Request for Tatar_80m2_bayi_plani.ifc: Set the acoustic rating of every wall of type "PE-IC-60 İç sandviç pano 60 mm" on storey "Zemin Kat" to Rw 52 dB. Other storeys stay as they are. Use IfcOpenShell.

First a look at what the model holds.

```python
import ifcopenshell
import ifcopenshell.util.element

model = ifcopenshell.open("Tatar_80m2_bayi_plani.ifc")
print(model.schema)
storey = next(s for s in model.by_type("IfcBuildingStorey") if s.Name == "Zemin Kat")
walls = [e for e in ifcopenshell.util.element.get_decomposition(storey) if e.is_a("IfcWall")]
seen = {}
for e in walls:
    element_type = ifcopenshell.util.element.get_type(e)
    key = (element_type.Name if element_type != e and element_type else None, ifcopenshell.util.element.get_pset(e, "Pset_WallCommon", "AcousticRating"))
    seen[key] = seen.get(key, 0) + 1
for (name, value), count in sorted(seen.items(), key=str):
    print(count, "x", name, "|", value)
```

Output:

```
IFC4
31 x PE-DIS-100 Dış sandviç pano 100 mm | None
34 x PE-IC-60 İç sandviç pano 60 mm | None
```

```python
import ifcopenshell
import ifcopenshell.api.pset
import ifcopenshell.util.element

model = ifcopenshell.open("Tatar_80m2_bayi_plani.ifc")

storey = next(s for s in model.by_type("IfcBuildingStorey") if s.Name == "Zemin Kat")
walls = [e for e in ifcopenshell.util.element.get_decomposition(storey) if e.is_a("IfcWall")]

count = 0
for e in walls:
    element_type = ifcopenshell.util.element.get_type(e)
    if element_type in (None, e) or element_type.Name != "PE-IC-60 İç sandviç pano 60 mm":
        continue
    # add_pset returns the element's existing set when there is one.
    pset = ifcopenshell.api.pset.add_pset(model, product=e, name="Pset_WallCommon")
    ifcopenshell.api.pset.edit_pset(model, pset=pset, properties={"AcousticRating": "Rw 52 dB"})
    count += 1

print(count, "walls updated")

model.write("Tatar_80m2_bayi_plani_edited.ifc")
```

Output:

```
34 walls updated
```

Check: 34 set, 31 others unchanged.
